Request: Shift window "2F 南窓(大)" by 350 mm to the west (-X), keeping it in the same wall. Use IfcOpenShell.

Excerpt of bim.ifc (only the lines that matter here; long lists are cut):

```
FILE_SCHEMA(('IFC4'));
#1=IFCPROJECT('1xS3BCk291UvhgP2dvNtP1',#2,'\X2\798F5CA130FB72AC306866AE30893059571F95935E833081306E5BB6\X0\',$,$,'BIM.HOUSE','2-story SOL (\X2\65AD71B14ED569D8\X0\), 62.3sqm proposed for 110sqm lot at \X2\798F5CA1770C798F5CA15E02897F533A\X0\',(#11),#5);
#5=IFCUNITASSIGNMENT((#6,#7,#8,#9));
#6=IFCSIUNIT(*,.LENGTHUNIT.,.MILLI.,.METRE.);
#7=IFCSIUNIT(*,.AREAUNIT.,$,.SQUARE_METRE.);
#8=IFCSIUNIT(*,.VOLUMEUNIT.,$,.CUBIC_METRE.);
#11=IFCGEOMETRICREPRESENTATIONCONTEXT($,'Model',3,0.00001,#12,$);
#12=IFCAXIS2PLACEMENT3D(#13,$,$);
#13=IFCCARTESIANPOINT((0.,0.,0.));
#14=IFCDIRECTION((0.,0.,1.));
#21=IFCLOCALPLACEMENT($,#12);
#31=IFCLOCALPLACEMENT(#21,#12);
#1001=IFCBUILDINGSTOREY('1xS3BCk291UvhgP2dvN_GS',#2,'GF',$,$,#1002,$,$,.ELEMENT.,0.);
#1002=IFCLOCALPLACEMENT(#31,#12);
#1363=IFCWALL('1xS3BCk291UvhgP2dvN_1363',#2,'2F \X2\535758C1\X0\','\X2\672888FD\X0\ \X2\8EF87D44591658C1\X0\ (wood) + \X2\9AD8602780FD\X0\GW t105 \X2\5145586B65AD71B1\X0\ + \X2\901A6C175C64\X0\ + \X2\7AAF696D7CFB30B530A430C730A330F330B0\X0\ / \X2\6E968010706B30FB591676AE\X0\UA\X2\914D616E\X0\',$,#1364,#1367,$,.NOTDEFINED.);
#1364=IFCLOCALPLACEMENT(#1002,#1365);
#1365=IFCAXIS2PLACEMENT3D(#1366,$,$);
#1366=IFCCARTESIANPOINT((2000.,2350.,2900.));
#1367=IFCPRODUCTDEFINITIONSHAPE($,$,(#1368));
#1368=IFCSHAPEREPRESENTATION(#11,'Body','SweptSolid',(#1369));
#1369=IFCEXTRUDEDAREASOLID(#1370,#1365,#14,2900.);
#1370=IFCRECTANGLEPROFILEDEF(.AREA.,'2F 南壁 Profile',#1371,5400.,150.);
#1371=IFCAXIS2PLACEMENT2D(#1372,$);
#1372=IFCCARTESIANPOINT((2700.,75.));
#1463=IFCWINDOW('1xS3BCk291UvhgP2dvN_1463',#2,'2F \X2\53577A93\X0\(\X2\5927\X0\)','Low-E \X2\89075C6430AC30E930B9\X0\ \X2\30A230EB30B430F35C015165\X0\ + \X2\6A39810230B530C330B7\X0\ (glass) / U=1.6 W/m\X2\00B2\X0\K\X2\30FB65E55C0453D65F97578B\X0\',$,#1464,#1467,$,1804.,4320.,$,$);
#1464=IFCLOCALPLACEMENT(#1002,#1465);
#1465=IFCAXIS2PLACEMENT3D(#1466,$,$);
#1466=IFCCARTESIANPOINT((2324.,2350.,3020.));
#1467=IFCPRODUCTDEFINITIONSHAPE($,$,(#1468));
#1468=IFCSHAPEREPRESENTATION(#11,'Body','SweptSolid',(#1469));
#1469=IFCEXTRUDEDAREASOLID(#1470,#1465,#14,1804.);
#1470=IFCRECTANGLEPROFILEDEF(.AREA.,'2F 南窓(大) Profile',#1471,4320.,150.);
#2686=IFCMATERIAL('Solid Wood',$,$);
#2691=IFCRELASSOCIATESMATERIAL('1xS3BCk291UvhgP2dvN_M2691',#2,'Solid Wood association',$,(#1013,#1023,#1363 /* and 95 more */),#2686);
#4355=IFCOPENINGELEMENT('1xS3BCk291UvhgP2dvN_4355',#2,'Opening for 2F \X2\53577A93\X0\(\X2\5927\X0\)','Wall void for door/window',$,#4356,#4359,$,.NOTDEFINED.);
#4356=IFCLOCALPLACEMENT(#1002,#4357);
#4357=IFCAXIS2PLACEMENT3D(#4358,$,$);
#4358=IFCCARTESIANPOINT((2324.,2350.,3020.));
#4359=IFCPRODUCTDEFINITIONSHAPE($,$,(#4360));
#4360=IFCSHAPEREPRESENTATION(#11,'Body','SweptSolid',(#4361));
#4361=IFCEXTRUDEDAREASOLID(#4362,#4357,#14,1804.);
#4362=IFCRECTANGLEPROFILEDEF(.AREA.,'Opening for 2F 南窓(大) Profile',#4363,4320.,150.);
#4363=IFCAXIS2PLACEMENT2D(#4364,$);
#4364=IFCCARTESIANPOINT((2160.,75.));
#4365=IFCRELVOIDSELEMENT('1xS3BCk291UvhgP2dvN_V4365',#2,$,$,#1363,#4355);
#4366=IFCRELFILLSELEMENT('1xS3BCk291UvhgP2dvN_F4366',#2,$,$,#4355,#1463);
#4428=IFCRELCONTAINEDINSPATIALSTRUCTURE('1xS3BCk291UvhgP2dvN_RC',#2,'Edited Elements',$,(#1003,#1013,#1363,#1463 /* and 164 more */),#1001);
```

```python
import ifcopenshell
import ifcopenshell.api.geometry
import ifcopenshell.util.placement
import ifcopenshell.util.unit

model = ifcopenshell.open("bim.ifc")
unit_scale = ifcopenshell.util.unit.calculate_unit_scale(model)

window = model.by_guid("1xS3BCk291UvhgP2dvN_1463")
opening = window.FillsVoids[0].RelatingOpeningElement
wall = opening.VoidsElements[0].RelatingBuildingElement

wall_matrix = ifcopenshell.util.placement.get_local_placement(wall.ObjectPlacement)
shift = wall_matrix[:3, 0] * -0.35 / unit_scale
before = ifcopenshell.util.placement.get_local_placement(window.ObjectPlacement)[:3, 3].copy()

# The window is not placed relative to its opening, so move both.
for product in (opening, window):
    matrix = ifcopenshell.util.placement.get_local_placement(product.ObjectPlacement)
    matrix[:3, 3] += shift
    ifcopenshell.api.geometry.edit_object_placement(model, product=product, matrix=matrix, is_si=False)

after = ifcopenshell.util.placement.get_local_placement(window.ObjectPlacement)[:3, 3]
print("window moved by", (after - before).round(3) + 0.0)

model.write("bim_edited.ifc")
```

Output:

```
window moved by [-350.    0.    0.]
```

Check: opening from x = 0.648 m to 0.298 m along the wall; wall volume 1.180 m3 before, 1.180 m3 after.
